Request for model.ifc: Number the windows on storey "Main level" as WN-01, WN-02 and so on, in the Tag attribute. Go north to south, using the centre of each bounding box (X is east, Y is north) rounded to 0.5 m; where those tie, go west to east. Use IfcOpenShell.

First a look at what the model holds.

```python
import ifcopenshell
import ifcopenshell.util.element
import ifcopenshell.util.placement

model = ifcopenshell.open("model.ifc")
print(model.schema)
storey = next(s for s in model.by_type("IfcBuildingStorey") if s.Name == "Main level")
windows = [e for e in ifcopenshell.util.element.get_decomposition(storey) if e.is_a("IfcWindow")]
for e in sorted(windows, key=lambda e: e.id()):
    origin = ifcopenshell.util.placement.get_local_placement(e.ObjectPlacement)[:3, 3]
    print(e.id(), e.Tag, e.Name, origin.round(2) + 0.0, sep=" | ")
```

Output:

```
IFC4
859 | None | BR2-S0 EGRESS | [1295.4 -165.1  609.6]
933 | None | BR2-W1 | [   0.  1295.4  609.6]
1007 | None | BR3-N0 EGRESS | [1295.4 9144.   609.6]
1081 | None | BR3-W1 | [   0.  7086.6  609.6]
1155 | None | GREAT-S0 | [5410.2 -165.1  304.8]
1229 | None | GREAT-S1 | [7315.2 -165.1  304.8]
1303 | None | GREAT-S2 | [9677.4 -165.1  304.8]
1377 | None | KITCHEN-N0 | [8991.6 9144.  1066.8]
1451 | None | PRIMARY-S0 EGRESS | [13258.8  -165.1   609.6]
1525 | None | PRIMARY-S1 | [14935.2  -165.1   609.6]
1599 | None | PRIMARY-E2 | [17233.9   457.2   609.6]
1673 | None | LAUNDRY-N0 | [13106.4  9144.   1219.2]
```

```python
import ifcopenshell
import ifcopenshell.geom
import ifcopenshell.util.element
import ifcopenshell.util.shape

model = ifcopenshell.open("model.ifc")
settings = ifcopenshell.geom.settings()
settings.set("use-world-coords", True)


def centre(element):
    shape = ifcopenshell.geom.create_shape(settings, element)
    return ifcopenshell.util.shape.get_bbox_centroid(shape.geometry)


storey = next(s for s in model.by_type("IfcBuildingStorey") if s.Name == "Main level")
windows = [e for e in ifcopenshell.util.element.get_decomposition(storey) if e.is_a("IfcWindow")]

# Insertion points can sit at a corner or the storey origin, so sort by the geometry (in metres).
centres = {e: centre(e) for e in windows}
windows.sort(key=lambda e: (-round(centres[e][1] / 0.5), centres[e][0]))

for i, e in enumerate(windows, start=1):
    number = f"WN-{i:02d}"
    e.Tag = number
    print(e.id(), number)

model.write("model_v2.ifc")
```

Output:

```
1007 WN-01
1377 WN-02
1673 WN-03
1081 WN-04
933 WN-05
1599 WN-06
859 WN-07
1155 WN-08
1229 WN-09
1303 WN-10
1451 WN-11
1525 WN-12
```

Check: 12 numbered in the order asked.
